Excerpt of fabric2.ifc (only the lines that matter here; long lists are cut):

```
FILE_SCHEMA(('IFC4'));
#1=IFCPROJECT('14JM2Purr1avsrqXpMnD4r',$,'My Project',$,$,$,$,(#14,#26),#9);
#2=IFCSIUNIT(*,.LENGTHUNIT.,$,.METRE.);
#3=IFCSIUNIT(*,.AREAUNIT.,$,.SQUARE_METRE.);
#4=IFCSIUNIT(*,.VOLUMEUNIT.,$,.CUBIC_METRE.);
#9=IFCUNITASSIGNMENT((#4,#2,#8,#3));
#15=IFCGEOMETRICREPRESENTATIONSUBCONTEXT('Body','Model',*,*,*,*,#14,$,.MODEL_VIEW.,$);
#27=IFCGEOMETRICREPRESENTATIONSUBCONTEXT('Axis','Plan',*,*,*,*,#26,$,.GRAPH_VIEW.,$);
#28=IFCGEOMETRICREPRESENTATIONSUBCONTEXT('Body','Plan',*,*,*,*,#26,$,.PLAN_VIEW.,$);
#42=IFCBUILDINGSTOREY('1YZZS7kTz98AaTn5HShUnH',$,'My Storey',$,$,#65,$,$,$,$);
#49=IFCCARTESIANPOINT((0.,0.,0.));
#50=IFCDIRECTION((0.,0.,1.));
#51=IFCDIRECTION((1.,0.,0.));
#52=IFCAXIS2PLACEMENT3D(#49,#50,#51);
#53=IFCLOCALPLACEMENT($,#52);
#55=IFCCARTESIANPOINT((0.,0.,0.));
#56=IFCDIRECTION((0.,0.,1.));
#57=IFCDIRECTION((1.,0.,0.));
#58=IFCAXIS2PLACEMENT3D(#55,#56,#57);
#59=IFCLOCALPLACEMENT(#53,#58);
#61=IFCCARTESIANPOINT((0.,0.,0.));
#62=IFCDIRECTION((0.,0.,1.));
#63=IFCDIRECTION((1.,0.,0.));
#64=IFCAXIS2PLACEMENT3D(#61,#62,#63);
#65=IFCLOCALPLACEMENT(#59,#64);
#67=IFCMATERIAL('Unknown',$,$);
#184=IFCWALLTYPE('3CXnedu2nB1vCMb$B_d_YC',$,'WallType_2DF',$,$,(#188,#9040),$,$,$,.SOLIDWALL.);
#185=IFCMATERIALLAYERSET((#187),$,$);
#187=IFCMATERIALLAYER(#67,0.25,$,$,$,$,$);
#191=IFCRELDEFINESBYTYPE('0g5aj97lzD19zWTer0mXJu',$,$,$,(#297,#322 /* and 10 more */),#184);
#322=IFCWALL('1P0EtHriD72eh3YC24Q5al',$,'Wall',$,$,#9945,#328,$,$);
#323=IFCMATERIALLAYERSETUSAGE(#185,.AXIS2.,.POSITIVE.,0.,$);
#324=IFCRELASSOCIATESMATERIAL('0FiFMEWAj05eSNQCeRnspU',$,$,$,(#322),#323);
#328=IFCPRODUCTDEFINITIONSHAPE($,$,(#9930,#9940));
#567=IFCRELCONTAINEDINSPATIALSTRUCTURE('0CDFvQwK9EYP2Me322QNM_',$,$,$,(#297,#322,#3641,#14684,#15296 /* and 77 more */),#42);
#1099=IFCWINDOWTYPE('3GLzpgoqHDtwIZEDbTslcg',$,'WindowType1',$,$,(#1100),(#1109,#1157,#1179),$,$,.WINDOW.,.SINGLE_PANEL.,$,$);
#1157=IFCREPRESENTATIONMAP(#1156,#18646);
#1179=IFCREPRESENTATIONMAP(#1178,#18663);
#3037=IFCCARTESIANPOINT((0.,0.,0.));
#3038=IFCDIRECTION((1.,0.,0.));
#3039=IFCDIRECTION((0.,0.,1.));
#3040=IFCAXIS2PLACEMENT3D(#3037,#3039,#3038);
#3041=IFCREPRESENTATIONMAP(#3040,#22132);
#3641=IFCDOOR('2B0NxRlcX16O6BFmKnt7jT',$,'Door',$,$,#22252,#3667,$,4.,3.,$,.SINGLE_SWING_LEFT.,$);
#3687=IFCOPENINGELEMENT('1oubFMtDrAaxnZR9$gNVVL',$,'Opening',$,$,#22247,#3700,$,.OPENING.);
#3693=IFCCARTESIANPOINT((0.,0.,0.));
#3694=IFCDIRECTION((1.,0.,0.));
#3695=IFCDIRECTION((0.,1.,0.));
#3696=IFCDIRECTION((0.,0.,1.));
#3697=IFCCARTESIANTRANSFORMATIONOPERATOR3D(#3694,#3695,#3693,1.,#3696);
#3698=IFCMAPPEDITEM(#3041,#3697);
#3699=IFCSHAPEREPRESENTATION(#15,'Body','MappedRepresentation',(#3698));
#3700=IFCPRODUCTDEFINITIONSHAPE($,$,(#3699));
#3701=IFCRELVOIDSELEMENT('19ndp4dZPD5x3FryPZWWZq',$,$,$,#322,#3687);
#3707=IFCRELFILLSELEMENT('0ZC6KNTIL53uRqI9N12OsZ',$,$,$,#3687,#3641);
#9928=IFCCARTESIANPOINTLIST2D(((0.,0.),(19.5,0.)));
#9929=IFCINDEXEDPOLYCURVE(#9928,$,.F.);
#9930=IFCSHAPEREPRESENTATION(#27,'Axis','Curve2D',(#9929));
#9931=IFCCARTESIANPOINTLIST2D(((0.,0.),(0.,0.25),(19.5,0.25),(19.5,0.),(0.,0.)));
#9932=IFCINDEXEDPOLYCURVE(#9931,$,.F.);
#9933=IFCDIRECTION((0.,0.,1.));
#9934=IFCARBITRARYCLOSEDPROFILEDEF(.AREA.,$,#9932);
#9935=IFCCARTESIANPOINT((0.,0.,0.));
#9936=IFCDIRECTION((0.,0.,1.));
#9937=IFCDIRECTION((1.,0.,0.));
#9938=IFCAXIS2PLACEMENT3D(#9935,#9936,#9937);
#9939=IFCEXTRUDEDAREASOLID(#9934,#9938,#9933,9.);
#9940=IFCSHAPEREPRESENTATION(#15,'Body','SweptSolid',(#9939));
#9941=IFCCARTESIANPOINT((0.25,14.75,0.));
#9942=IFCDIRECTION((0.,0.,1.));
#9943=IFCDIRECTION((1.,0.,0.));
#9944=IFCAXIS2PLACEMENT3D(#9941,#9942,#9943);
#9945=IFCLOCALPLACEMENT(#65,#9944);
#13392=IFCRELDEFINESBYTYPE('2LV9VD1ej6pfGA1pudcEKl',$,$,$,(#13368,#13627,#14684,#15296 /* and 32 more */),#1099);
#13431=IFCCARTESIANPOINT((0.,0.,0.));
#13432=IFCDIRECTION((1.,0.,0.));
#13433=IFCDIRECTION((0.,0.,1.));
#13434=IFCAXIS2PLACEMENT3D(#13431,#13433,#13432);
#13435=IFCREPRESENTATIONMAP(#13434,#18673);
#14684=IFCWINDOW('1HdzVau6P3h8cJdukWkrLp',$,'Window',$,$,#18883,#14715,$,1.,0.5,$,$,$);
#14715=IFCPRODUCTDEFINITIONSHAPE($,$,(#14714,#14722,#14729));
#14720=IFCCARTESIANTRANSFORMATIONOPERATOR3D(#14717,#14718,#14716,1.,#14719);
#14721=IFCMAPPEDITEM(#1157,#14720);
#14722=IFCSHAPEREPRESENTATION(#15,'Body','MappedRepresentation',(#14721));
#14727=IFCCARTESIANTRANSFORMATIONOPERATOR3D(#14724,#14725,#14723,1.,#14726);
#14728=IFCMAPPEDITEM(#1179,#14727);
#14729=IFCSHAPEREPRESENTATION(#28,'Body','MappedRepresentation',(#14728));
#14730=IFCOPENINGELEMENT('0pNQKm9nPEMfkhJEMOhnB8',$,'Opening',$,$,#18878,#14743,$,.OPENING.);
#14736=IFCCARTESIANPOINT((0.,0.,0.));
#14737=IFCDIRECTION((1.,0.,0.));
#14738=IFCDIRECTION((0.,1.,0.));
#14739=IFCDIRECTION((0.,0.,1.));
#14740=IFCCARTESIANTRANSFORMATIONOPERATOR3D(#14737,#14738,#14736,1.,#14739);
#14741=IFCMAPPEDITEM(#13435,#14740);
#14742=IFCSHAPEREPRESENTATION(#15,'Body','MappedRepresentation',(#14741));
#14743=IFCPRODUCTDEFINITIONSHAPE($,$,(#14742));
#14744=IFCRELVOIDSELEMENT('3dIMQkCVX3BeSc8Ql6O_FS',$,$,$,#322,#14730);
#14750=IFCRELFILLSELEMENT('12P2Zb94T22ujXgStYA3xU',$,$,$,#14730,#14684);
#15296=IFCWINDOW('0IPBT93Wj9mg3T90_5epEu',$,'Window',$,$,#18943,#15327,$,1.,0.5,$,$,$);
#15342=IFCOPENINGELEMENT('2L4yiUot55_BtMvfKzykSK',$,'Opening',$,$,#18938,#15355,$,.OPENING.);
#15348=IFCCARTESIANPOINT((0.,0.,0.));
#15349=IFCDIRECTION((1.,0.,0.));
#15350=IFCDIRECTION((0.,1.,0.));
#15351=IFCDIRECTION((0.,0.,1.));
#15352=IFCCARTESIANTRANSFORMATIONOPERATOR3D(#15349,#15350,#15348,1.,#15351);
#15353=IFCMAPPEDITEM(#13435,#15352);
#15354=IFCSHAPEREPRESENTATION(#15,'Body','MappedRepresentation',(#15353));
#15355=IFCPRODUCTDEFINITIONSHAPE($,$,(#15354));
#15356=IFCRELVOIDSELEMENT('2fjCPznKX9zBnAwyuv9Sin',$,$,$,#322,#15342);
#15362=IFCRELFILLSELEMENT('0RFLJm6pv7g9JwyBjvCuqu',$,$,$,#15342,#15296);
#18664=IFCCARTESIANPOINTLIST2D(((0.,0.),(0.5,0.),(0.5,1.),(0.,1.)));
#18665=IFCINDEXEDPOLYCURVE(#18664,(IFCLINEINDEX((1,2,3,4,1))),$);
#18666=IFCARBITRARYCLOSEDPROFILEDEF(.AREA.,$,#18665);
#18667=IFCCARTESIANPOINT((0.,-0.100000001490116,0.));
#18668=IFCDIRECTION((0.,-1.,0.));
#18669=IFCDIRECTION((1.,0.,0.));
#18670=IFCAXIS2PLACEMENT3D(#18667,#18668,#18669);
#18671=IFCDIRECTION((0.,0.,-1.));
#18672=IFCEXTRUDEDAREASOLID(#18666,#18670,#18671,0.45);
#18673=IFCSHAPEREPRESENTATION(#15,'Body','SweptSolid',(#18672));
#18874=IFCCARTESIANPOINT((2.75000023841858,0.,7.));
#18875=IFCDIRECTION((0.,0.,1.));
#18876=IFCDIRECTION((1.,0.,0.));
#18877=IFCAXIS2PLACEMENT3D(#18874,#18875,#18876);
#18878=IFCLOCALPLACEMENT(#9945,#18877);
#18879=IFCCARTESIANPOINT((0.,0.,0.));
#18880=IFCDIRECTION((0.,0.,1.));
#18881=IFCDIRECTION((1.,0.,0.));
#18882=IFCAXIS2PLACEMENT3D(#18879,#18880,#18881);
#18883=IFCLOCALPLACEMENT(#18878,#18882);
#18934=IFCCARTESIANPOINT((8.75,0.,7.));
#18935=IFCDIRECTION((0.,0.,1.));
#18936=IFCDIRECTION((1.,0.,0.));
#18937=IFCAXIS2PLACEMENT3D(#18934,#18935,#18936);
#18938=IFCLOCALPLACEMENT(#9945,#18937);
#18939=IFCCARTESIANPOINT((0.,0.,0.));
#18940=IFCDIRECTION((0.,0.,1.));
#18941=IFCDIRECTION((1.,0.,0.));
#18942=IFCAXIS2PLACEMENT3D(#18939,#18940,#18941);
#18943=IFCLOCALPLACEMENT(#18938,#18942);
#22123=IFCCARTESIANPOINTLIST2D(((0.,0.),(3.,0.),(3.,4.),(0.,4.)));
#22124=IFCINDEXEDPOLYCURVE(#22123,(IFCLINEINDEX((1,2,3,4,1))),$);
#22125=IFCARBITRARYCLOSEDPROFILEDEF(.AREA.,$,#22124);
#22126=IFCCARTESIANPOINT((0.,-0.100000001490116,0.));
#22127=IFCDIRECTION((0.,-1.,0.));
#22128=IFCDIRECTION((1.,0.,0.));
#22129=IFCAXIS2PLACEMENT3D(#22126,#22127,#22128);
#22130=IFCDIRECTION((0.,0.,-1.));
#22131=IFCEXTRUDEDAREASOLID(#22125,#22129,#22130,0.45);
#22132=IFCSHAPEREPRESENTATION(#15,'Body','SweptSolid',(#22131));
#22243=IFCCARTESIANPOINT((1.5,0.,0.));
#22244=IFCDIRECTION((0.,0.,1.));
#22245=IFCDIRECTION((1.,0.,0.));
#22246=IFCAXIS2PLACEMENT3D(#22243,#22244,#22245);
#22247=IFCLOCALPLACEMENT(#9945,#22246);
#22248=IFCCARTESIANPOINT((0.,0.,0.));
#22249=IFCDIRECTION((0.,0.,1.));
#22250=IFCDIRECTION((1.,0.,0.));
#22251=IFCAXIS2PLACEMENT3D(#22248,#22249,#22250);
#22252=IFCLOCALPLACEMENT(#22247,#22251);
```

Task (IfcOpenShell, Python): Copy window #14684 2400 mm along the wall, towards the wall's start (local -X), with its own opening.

```python
import ifcopenshell
import ifcopenshell.api.feature
import ifcopenshell.api.geometry
import ifcopenshell.api.root
import ifcopenshell.geom
import ifcopenshell.util.element
import ifcopenshell.util.placement
import ifcopenshell.util.shape
import ifcopenshell.util.unit

model = ifcopenshell.open("fabric2.ifc")
unit_scale = ifcopenshell.util.unit.calculate_unit_scale(model)
settings = ifcopenshell.geom.settings()


def volume(element):
    """Net volume in cubic metres, openings subtracted."""
    shape = ifcopenshell.geom.create_shape(settings, element)
    return ifcopenshell.util.shape.get_volume(shape.geometry)


window = model.by_id(14684)
opening = window.FillsVoids[0].RelatingOpeningElement
wall = opening.VoidsElements[0].RelatingBuildingElement
before = volume(wall)
shift = ifcopenshell.util.placement.get_local_placement(wall.ObjectPlacement)[:3, 0] * -2.4 / unit_scale

# copy_class copies the void relationship, type, container and properties, but no geometry.
new_opening = ifcopenshell.api.root.copy_class(model, product=opening)
new_opening.Representation = ifcopenshell.util.element.copy_deep(
    model, opening.Representation, exclude=["IfcGeometricRepresentationContext", "IfcRepresentationMap"]
)
new_window = ifcopenshell.api.root.copy_class(model, product=window)
new_window.Representation = ifcopenshell.util.element.copy_deep(
    model, window.Representation, exclude=["IfcGeometricRepresentationContext", "IfcRepresentationMap"]
)
ifcopenshell.api.feature.add_filling(model, opening=new_opening, element=new_window)

for old, new in ((opening, new_opening), (window, new_window)):
    matrix = ifcopenshell.util.placement.get_local_placement(old.ObjectPlacement)
    matrix[:3, 3] += shift
    ifcopenshell.api.geometry.edit_object_placement(model, product=new, matrix=matrix, is_si=False)

after = volume(wall)

print(f"wall volume {before:.3f} -> {after:.3f} m3")

model.write("fabric2_edited.ifc")
```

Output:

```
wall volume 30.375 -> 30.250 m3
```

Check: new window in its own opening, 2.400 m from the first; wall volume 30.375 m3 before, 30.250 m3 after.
